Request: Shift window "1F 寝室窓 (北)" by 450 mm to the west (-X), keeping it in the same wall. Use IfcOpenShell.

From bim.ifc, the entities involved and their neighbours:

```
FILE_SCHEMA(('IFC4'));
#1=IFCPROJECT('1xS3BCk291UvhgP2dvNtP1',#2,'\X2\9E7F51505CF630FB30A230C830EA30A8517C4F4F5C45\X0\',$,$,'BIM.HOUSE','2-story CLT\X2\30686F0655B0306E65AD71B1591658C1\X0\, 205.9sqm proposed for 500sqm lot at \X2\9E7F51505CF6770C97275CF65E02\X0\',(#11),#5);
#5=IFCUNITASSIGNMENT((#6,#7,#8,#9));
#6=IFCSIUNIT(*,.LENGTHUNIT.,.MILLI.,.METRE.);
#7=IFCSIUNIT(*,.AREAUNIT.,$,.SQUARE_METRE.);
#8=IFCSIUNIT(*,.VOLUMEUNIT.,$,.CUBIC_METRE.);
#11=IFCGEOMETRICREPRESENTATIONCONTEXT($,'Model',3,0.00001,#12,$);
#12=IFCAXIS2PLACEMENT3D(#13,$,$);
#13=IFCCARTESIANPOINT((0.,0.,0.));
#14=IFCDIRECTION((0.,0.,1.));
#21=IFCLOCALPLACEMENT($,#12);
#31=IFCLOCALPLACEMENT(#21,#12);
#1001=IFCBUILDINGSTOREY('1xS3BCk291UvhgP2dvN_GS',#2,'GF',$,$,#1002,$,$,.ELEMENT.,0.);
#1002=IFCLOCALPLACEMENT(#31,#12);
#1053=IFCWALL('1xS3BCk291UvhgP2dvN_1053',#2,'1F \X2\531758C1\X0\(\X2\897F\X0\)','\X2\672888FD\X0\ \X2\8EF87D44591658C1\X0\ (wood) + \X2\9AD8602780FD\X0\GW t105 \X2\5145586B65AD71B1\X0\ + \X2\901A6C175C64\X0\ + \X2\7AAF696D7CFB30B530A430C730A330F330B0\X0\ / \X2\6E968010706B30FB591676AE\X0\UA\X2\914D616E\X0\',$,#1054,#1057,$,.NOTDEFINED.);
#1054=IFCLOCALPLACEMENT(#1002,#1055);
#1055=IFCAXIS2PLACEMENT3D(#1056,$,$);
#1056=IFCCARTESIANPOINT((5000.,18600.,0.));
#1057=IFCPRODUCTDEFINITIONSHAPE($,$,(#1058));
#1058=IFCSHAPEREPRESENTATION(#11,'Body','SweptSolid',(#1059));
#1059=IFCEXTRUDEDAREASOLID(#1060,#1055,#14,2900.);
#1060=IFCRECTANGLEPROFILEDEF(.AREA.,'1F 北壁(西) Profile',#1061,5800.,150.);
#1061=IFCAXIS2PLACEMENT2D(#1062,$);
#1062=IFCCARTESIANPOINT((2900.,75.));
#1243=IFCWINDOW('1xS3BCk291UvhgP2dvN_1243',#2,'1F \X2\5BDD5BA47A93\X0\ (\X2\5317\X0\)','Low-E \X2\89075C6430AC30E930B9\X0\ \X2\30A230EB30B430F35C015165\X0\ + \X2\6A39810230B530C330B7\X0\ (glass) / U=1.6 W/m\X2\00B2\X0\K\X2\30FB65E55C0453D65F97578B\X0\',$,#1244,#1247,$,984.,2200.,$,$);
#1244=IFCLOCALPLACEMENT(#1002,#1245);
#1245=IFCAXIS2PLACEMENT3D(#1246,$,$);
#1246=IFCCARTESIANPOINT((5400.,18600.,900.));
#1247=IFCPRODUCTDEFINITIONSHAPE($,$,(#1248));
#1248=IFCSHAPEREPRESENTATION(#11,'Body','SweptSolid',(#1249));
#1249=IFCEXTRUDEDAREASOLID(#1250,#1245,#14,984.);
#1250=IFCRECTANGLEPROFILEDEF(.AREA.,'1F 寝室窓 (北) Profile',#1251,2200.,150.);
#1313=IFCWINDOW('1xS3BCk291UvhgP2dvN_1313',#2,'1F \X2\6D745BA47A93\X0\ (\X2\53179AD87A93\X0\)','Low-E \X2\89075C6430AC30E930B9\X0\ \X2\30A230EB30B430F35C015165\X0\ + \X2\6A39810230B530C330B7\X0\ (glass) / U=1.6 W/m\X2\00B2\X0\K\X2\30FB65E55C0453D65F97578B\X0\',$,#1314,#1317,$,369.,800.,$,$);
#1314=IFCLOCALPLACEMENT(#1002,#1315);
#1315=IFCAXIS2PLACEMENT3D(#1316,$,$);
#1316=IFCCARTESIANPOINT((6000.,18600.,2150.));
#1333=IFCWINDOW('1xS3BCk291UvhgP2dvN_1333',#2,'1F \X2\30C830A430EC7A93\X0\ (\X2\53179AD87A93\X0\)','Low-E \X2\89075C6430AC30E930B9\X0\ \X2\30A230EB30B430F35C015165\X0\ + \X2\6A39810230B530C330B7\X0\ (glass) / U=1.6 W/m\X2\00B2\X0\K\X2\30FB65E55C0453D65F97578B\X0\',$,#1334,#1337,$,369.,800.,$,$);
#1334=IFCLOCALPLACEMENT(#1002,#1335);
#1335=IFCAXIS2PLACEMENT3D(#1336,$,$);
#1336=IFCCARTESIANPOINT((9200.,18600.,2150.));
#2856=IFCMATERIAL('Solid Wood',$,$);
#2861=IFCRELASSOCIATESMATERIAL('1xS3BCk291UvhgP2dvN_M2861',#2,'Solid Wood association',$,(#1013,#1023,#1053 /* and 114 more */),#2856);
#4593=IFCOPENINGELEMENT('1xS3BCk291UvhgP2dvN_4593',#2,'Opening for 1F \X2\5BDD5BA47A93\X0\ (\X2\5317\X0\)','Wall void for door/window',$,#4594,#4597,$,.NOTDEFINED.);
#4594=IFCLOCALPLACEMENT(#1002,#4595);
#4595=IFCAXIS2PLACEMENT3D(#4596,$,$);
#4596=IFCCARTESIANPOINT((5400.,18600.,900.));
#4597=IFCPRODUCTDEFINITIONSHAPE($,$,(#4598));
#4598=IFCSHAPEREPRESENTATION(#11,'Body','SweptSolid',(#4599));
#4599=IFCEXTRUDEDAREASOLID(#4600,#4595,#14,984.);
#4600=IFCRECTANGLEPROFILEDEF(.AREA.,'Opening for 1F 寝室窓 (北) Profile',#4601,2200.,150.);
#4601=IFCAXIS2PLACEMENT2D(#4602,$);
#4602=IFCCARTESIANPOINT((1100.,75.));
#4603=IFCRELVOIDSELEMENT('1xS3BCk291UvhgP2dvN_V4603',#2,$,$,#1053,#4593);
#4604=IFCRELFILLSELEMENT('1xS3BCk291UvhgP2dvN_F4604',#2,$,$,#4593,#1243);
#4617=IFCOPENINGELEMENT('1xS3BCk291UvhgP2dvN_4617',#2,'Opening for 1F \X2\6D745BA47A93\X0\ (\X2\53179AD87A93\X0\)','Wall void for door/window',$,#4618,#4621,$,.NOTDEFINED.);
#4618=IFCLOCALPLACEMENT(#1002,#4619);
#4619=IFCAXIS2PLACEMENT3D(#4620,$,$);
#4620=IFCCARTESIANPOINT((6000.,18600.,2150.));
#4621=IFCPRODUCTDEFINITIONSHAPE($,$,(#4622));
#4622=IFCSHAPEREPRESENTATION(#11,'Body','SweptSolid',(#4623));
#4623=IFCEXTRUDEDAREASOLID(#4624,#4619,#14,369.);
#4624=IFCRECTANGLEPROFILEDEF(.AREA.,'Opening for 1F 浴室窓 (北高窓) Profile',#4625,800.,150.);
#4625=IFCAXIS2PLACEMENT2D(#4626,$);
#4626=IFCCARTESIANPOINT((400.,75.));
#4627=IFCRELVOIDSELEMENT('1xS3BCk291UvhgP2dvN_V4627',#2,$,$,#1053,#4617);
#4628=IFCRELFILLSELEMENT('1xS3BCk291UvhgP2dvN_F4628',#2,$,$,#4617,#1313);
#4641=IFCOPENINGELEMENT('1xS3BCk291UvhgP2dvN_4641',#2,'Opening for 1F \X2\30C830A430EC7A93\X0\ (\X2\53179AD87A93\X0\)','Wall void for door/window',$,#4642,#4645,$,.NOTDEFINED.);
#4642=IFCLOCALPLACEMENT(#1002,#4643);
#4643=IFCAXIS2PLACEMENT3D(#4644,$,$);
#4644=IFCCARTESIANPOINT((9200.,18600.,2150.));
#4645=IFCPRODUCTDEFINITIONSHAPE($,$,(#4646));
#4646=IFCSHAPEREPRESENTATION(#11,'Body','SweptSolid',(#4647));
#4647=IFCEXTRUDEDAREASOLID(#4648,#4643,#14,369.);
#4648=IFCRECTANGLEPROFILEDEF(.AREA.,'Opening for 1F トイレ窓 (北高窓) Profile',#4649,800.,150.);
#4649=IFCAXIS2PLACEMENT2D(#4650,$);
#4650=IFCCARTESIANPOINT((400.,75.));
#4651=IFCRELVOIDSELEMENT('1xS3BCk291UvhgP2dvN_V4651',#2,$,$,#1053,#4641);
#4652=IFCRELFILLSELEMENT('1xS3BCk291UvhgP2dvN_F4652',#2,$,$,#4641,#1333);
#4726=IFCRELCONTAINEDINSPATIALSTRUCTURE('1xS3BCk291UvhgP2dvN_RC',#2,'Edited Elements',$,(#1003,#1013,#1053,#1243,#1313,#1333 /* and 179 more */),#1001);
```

```python
import ifcopenshell
import ifcopenshell.api.geometry
import ifcopenshell.util.placement
import ifcopenshell.util.unit

model = ifcopenshell.open("bim.ifc")
unit_scale = ifcopenshell.util.unit.calculate_unit_scale(model)

window = model.by_guid("1xS3BCk291UvhgP2dvN_1243")
opening = window.FillsVoids[0].RelatingOpeningElement
wall = opening.VoidsElements[0].RelatingBuildingElement

wall_matrix = ifcopenshell.util.placement.get_local_placement(wall.ObjectPlacement)
shift = wall_matrix[:3, 0] * -0.45 / unit_scale
before = ifcopenshell.util.placement.get_local_placement(window.ObjectPlacement)[:3, 3].copy()

# The window is not placed relative to its opening, so move both.
for product in (opening, window):
    matrix = ifcopenshell.util.placement.get_local_placement(product.ObjectPlacement)
    matrix[:3, 3] += shift
    ifcopenshell.api.geometry.edit_object_placement(model, product=product, matrix=matrix, is_si=False)

after = ifcopenshell.util.placement.get_local_placement(window.ObjectPlacement)[:3, 3]
print("window moved by", (after - before).round(3) + 0.0)

model.write("bim-out.ifc")
```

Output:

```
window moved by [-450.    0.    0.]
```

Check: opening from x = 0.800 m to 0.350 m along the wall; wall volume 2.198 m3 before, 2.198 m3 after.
